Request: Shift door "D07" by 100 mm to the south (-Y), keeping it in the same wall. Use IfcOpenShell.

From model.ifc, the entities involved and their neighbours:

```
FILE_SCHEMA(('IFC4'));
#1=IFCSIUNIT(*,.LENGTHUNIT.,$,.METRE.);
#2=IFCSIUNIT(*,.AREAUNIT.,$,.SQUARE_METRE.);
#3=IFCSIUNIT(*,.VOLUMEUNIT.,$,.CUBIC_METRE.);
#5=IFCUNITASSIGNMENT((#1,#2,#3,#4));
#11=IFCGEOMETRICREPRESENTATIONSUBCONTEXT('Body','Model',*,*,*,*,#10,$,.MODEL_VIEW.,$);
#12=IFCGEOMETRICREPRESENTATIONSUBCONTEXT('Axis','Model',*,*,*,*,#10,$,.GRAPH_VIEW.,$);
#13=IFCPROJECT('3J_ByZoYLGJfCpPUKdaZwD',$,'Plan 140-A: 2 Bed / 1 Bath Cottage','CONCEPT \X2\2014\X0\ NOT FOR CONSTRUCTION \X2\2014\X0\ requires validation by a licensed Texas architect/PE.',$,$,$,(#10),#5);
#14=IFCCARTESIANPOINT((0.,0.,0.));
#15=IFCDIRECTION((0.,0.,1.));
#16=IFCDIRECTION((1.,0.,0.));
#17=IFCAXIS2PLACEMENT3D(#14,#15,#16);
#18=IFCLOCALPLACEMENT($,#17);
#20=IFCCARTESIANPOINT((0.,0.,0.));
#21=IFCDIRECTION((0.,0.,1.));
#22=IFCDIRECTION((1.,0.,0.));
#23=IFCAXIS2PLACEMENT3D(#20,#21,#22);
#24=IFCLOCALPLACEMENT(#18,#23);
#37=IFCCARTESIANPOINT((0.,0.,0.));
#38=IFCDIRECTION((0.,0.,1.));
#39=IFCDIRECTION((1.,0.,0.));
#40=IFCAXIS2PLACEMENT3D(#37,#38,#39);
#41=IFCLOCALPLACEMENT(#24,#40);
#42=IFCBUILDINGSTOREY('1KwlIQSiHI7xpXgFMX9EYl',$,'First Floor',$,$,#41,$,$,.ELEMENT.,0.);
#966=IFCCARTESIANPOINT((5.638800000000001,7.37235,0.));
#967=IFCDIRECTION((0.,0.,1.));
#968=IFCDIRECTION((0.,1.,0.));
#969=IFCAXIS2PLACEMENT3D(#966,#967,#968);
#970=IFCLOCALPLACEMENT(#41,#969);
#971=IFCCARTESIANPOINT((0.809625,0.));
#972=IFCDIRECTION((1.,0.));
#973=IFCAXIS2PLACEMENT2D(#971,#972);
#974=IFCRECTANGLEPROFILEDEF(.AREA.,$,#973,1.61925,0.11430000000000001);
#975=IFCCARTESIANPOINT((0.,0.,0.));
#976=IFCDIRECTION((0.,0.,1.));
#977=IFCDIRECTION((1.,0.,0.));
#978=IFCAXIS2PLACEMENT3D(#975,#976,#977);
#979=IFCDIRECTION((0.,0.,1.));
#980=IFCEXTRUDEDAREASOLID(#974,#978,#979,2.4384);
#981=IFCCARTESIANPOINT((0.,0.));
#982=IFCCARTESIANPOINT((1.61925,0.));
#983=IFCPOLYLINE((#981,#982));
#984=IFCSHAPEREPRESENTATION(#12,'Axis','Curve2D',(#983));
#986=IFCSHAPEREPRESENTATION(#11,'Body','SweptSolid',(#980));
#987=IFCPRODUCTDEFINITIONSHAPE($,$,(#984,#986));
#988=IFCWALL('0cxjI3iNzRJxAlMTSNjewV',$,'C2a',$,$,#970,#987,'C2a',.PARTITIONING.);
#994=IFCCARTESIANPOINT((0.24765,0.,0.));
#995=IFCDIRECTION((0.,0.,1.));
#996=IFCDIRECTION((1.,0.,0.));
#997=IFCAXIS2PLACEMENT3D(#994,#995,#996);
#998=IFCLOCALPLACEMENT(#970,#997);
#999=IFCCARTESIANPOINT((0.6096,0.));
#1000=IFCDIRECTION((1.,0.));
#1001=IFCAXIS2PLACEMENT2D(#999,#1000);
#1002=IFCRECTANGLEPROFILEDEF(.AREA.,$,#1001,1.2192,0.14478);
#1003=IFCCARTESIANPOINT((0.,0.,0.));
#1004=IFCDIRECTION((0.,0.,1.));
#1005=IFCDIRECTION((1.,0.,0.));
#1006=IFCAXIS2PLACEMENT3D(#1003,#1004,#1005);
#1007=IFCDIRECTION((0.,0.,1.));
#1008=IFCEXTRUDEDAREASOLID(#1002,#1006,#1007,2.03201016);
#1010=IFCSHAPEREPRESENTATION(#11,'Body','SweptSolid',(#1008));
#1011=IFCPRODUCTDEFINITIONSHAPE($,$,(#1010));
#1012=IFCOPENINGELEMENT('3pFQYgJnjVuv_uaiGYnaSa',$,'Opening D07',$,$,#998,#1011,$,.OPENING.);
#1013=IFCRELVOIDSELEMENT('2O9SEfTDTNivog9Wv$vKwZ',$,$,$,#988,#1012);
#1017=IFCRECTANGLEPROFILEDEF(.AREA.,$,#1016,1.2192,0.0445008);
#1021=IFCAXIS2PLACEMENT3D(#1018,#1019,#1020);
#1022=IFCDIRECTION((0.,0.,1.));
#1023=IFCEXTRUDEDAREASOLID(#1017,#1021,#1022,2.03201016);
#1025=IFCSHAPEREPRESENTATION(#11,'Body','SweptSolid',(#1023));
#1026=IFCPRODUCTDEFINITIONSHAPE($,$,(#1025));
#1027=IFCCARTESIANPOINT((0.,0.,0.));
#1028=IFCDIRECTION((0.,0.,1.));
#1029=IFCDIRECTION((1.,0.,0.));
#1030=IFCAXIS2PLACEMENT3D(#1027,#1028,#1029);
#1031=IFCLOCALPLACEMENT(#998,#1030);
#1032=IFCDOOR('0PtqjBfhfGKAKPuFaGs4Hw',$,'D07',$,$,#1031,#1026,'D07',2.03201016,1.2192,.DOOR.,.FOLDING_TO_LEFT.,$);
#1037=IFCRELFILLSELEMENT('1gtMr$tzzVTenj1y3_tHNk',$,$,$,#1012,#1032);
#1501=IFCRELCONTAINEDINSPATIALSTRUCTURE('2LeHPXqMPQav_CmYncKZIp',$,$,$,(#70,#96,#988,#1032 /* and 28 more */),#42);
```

```python
import ifcopenshell
import ifcopenshell.api.geometry
import ifcopenshell.util.placement
import ifcopenshell.util.unit

model = ifcopenshell.open("model.ifc")
unit_scale = ifcopenshell.util.unit.calculate_unit_scale(model)

door = model.by_id(1032)
opening = door.FillsVoids[0].RelatingOpeningElement
wall = opening.VoidsElements[0].RelatingBuildingElement

wall_matrix = ifcopenshell.util.placement.get_local_placement(wall.ObjectPlacement)
shift = wall_matrix[:3, 0] * -0.1 / unit_scale
before = ifcopenshell.util.placement.get_local_placement(door.ObjectPlacement)[:3, 3].copy()

# The door is placed relative to its opening, so it follows when the opening moves.
matrix = ifcopenshell.util.placement.get_local_placement(opening.ObjectPlacement)
matrix[:3, 3] += shift
ifcopenshell.api.geometry.edit_object_placement(
    model, product=opening, matrix=matrix, is_si=False, should_transform_children=True
)

after = ifcopenshell.util.placement.get_local_placement(door.ObjectPlacement)[:3, 3]
print("door moved by", (after - before).round(3) + 0.0)

model.write("model_v2.ifc")
```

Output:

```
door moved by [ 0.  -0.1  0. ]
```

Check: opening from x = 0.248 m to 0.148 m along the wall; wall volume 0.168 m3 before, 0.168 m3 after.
